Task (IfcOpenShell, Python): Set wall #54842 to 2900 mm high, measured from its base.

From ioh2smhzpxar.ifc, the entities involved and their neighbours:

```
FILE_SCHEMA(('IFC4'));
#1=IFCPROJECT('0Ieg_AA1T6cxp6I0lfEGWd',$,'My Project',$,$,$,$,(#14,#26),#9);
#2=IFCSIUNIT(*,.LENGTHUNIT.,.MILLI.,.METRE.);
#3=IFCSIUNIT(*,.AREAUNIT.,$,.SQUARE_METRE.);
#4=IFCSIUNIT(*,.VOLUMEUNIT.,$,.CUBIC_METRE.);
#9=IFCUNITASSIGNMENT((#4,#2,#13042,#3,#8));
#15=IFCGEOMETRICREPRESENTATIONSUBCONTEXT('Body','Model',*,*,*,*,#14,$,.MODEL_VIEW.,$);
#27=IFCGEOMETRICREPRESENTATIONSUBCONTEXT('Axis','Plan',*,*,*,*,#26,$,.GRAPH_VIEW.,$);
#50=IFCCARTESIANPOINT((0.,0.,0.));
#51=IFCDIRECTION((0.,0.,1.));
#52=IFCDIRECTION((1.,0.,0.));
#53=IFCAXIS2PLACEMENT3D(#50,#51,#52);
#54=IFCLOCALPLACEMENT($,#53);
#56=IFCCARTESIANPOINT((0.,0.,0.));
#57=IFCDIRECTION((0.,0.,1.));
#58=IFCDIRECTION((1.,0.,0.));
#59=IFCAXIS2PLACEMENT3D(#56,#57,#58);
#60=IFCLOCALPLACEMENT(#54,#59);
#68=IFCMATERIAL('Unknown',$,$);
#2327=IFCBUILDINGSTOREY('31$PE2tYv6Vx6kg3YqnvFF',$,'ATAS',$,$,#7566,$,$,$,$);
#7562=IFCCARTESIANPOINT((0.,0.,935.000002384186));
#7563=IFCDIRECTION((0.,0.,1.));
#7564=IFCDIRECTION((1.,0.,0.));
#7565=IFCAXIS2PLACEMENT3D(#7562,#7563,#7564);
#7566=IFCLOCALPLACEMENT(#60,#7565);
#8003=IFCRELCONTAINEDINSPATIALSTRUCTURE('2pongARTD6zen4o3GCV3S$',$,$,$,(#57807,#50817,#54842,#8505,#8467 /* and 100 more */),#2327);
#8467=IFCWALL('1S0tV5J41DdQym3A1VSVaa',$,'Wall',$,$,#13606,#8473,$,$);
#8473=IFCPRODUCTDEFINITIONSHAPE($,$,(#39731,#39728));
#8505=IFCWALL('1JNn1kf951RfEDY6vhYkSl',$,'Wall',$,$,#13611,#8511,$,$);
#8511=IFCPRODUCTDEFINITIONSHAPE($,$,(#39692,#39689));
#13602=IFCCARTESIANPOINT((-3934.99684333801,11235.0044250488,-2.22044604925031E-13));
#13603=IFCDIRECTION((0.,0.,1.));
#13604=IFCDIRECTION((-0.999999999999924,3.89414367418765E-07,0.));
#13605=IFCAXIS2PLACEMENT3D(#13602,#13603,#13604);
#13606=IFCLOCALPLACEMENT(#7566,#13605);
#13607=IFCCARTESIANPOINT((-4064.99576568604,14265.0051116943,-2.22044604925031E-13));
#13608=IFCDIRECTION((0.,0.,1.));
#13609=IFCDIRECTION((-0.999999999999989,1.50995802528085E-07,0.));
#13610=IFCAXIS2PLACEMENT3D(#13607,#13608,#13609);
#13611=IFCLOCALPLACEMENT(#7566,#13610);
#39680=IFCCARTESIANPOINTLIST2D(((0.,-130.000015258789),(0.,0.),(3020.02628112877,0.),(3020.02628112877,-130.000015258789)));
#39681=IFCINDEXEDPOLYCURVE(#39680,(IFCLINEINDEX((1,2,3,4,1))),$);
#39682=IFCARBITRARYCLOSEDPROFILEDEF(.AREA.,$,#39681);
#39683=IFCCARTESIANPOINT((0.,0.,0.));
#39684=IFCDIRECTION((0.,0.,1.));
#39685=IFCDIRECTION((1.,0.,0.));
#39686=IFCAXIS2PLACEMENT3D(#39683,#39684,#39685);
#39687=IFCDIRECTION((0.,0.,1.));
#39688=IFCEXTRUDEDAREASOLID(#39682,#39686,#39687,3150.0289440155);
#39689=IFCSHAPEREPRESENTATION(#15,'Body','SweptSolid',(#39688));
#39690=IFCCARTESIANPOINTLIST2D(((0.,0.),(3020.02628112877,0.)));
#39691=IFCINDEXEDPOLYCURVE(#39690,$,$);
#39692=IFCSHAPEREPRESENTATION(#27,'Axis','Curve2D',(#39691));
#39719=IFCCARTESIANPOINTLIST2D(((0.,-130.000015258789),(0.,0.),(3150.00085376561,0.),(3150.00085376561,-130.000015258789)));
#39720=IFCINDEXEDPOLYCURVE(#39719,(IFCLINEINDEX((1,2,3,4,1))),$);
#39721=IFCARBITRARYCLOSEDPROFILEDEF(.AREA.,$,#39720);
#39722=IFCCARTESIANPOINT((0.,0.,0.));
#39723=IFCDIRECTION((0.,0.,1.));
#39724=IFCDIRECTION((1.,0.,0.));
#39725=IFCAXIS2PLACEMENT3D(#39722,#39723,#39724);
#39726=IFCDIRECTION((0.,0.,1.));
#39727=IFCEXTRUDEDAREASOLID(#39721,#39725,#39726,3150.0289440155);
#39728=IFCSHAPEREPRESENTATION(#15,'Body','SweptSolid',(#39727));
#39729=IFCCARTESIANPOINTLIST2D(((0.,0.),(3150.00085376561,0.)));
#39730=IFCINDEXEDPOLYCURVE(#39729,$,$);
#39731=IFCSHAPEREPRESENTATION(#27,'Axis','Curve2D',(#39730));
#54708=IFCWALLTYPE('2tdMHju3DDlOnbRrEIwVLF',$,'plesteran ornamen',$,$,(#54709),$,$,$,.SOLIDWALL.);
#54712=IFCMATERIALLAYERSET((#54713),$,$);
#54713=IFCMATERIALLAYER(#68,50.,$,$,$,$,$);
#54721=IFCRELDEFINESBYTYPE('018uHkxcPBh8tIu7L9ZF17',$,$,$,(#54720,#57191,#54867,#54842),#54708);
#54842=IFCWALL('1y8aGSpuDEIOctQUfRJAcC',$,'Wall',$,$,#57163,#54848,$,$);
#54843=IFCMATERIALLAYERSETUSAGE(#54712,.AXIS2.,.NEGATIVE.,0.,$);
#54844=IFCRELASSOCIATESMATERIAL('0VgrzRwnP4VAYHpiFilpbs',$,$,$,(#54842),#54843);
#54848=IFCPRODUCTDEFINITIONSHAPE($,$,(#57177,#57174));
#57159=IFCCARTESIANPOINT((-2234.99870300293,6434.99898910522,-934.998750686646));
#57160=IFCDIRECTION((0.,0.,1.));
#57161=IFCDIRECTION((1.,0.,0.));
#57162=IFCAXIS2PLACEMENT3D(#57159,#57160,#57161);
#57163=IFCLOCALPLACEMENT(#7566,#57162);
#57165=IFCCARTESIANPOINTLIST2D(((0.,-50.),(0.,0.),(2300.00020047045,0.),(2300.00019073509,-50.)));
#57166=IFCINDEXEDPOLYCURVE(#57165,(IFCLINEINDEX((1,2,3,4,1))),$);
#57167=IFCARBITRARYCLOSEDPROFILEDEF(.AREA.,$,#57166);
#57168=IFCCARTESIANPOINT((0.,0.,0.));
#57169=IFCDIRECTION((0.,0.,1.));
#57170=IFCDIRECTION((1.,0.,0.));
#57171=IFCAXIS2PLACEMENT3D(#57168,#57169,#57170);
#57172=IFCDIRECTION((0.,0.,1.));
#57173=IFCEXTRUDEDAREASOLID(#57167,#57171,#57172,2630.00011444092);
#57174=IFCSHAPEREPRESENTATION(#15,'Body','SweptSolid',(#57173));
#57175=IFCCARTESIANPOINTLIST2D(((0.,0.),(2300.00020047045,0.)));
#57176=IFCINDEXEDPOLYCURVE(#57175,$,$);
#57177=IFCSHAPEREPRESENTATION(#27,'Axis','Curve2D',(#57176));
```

```python
import ifcopenshell
import ifcopenshell.geom
import ifcopenshell.util.representation
import ifcopenshell.util.shape
import ifcopenshell.util.unit

model = ifcopenshell.open("ioh2smhzpxar.ifc")
unit_scale = ifcopenshell.util.unit.calculate_unit_scale(model)
settings = ifcopenshell.geom.settings()


def volume(element):
    """Net volume in cubic metres, openings subtracted."""
    shape = ifcopenshell.geom.create_shape(settings, element)
    return ifcopenshell.util.shape.get_volume(shape.geometry)


wall = model.by_id(54842)
before = volume(wall)

body = ifcopenshell.util.representation.get_representation(wall, "Model", "Body")
solid = body.Items[0]
old_height = solid.Depth
solid.Depth = 2.9 / unit_scale
after = volume(wall)

print(f"height {old_height:g} -> {solid.Depth:g}, volume {before:.3f} -> {after:.3f} m3")

model.write("ioh2smhzpxar_updated.ifc")
```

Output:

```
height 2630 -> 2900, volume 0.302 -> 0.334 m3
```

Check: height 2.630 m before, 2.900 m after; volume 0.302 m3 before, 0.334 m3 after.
